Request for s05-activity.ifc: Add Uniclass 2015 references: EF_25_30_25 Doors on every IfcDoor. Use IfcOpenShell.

First a look at what the model holds.

```python
import ifcopenshell

model = ifcopenshell.open("s05-activity.ifc")
print(model.schema)
print("classifications:", [c.Name for c in model.by_type("IfcClassification")])
for ifc_class in ("IfcDoor", "IfcRoof", "IfcStair", "IfcWall", "IfcWindow"):
    print(ifc_class, len(model.by_type(ifc_class)))
```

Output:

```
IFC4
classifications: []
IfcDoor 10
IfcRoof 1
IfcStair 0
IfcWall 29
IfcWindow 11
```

```python
import ifcopenshell
import ifcopenshell.api.classification

model = ifcopenshell.open("s05-activity.ifc")

system = ifcopenshell.api.classification.add_classification(model, classification="Uniclass 2015")

codes = {
    "IfcDoor": ("EF_25_30_25", "Doors"),
}
for ifc_class, (code, name) in codes.items():
    products = model.by_type(ifc_class)
    ifcopenshell.api.classification.add_reference(
        model, products=products, classification=system, identification=code, name=name
    )
    print(code, len(products))

model.write("s05-activity_edited.ifc")
```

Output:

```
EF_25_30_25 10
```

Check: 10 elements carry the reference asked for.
